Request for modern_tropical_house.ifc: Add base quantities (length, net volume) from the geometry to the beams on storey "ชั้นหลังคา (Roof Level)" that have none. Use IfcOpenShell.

First a look at what the model holds.

```python
import ifcopenshell
import ifcopenshell.util.element
import ifcopenshell.util.unit

model = ifcopenshell.open("modern_tropical_house.ifc")
print(model.schema)
for unit_type in ("LENGTHUNIT", "AREAUNIT", "VOLUMEUNIT"):
    print(unit_type, ifcopenshell.util.unit.calculate_unit_scale(model, unit_type))
storey = next(s for s in model.by_type("IfcBuildingStorey") if s.Name == "ชั้นหลังคา (Roof Level)")
beams = [e for e in ifcopenshell.util.element.get_decomposition(storey) if e.is_a("IfcBeam")]
for e in sorted(beams, key=lambda e: e.id()):
    print(e.id(), e.is_a(), e.Name, list(ifcopenshell.util.element.get_psets(e, qtos_only=True)), sep=" | ")
```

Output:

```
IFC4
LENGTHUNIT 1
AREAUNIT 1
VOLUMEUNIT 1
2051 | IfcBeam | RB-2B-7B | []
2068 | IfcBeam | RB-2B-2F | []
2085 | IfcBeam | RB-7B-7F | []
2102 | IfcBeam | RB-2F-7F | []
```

```python
import ifcopenshell
import ifcopenshell.api.pset
import ifcopenshell.geom
import ifcopenshell.util.element
import ifcopenshell.util.shape
import ifcopenshell.util.unit

model = ifcopenshell.open("modern_tropical_house.ifc")
unit_scale = ifcopenshell.util.unit.calculate_unit_scale(model)
volume_scale = ifcopenshell.util.unit.calculate_unit_scale(model, "VOLUMEUNIT")
settings = ifcopenshell.geom.settings()

storey = next(s for s in model.by_type("IfcBuildingStorey") if s.Name == "ชั้นหลังคา (Roof Level)")
beams = [e for e in ifcopenshell.util.element.get_decomposition(storey) if e.is_a("IfcBeam")]

for e in sorted(beams, key=lambda e: e.id()):
    if ifcopenshell.util.element.get_psets(e, qtos_only=True, should_inherit=False):
        continue
    # Geometry comes back in metres, in the element's own axes.
    shape = ifcopenshell.geom.create_shape(settings, e)
    values = {
        "Length": ifcopenshell.util.shape.get_max_xyz(shape.geometry) / unit_scale,
        "NetVolume": ifcopenshell.util.shape.get_volume(shape.geometry) / volume_scale,
    }
    qto = ifcopenshell.api.pset.add_qto(model, product=e, name="Qto_BeamBaseQuantities")
    ifcopenshell.api.pset.edit_qto(model, qto=qto, properties=values)
    print(e.id(), {k: round(v, 3) for k, v in values.items()})

model.write("modern_tropical_house-out.ifc")
```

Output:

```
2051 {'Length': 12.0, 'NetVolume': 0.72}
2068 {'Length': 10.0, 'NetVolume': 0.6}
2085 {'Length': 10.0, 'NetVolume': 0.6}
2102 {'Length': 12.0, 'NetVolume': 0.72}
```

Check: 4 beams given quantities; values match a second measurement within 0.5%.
